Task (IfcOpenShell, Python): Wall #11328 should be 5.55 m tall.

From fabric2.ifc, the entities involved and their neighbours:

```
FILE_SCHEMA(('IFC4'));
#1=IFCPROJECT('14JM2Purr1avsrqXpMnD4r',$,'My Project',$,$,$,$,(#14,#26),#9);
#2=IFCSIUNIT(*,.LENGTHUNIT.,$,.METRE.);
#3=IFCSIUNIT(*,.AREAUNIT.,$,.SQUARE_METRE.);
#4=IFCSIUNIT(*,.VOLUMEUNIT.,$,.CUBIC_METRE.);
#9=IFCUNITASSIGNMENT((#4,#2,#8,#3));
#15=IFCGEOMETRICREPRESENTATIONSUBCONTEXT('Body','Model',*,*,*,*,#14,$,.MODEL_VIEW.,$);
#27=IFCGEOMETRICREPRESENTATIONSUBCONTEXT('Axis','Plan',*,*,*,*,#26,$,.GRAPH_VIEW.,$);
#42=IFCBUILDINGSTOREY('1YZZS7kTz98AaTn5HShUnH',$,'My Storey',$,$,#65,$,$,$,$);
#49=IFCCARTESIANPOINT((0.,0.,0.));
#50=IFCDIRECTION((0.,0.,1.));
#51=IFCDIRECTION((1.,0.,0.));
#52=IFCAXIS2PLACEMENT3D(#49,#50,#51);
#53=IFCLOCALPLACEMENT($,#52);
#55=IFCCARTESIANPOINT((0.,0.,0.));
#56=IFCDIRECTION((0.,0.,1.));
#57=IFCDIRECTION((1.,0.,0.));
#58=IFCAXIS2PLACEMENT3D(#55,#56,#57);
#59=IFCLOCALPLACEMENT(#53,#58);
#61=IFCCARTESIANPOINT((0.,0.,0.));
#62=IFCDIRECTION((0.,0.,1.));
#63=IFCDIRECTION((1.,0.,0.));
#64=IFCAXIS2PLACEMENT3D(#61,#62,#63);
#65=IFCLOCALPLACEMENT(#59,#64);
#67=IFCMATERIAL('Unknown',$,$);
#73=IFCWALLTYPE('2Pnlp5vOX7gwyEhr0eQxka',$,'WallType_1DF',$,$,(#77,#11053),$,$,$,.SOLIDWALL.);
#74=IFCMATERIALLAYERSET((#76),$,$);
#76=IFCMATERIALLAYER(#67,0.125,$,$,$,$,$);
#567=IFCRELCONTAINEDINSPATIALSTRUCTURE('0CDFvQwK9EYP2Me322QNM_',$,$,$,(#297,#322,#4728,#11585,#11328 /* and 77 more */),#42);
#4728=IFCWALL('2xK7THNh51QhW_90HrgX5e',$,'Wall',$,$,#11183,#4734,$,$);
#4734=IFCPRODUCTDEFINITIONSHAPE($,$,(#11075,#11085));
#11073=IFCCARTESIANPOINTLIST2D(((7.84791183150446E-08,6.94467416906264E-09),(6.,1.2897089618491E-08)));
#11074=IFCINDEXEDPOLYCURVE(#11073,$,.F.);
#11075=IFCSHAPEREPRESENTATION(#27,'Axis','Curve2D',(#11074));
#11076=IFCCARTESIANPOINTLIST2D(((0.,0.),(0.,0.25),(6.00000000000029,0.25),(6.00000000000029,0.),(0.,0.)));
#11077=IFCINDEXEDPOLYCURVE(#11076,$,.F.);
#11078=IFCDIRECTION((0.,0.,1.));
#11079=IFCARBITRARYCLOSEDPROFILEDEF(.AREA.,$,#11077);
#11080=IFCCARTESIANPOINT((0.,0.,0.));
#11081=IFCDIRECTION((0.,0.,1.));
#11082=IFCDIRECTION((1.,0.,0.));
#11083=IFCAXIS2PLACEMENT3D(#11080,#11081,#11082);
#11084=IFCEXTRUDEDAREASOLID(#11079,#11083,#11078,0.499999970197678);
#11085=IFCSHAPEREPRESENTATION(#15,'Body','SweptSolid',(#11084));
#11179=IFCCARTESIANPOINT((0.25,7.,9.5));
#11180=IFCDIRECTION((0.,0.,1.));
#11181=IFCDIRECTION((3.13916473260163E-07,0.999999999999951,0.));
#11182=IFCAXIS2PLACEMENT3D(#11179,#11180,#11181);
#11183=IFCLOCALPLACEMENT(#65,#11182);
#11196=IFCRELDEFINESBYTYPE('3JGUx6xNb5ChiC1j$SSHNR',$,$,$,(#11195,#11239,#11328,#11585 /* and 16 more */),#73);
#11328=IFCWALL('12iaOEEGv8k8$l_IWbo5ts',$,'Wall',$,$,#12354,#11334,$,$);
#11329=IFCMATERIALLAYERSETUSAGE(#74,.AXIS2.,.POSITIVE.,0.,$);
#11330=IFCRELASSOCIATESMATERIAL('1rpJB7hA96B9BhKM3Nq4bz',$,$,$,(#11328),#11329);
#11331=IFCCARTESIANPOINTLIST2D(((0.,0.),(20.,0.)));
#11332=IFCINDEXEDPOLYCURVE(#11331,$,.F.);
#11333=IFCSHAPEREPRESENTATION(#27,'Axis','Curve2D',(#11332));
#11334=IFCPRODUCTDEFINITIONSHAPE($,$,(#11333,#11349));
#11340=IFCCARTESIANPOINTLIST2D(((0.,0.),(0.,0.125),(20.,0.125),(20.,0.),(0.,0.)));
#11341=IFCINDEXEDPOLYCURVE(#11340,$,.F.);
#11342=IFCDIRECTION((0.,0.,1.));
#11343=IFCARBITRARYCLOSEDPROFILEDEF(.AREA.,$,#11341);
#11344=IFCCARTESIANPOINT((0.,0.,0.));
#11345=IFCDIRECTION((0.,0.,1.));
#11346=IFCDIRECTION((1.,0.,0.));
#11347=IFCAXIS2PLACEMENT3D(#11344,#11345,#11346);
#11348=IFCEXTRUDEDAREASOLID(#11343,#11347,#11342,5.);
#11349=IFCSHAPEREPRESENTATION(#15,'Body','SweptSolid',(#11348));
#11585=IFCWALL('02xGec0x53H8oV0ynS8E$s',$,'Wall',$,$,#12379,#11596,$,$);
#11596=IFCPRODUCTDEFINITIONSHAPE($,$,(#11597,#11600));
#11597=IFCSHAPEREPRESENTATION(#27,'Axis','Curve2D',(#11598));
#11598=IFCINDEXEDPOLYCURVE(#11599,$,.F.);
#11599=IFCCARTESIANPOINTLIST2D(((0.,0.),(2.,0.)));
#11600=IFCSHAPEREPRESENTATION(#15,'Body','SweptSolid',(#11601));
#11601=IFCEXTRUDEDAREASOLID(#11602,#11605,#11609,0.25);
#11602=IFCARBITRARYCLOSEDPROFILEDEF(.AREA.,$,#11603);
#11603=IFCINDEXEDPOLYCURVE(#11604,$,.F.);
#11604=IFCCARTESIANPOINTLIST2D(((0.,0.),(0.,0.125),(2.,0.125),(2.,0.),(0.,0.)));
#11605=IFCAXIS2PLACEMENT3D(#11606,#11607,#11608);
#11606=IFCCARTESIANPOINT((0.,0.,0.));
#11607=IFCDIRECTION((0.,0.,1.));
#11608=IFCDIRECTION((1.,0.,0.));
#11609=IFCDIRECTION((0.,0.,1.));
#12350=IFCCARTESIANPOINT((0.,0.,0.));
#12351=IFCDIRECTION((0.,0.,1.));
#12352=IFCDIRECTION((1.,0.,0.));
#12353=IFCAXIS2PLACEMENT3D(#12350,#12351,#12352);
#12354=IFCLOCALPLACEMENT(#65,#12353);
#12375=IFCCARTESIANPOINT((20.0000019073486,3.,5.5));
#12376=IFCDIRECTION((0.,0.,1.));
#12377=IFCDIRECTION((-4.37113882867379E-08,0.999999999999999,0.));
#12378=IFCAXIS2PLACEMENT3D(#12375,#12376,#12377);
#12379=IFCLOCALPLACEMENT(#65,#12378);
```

```python
import ifcopenshell
import ifcopenshell.geom
import ifcopenshell.util.representation
import ifcopenshell.util.shape
import ifcopenshell.util.unit

model = ifcopenshell.open("fabric2.ifc")
unit_scale = ifcopenshell.util.unit.calculate_unit_scale(model)
settings = ifcopenshell.geom.settings()


def volume(element):
    """Net volume in cubic metres, openings subtracted."""
    shape = ifcopenshell.geom.create_shape(settings, element)
    return ifcopenshell.util.shape.get_volume(shape.geometry)


wall = model.by_id(11328)
before = volume(wall)

body = ifcopenshell.util.representation.get_representation(wall, "Model", "Body")
solid = body.Items[0]
old_height = solid.Depth
solid.Depth = 5.55 / unit_scale
after = volume(wall)

print(f"height {old_height:g} -> {solid.Depth:g}, volume {before:.3f} -> {after:.3f} m3")

model.write("fabric2_rev.ifc")
```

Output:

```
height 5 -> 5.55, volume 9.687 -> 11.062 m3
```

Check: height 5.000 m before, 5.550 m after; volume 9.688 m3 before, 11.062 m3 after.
